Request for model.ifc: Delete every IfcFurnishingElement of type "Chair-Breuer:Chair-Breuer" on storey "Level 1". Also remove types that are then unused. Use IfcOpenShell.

First a look at what the model holds.

```python
import ifcopenshell
import ifcopenshell.util.element

model = ifcopenshell.open("model.ifc")
print(model.schema)
storey = next(s for s in model.by_type("IfcBuildingStorey") if s.Name == "Level 1")
furniture = [e for e in ifcopenshell.util.element.get_decomposition(storey) if e.is_a("IfcFurnishingElement")]
seen = {}
for e in furniture:
    element_type = ifcopenshell.util.element.get_type(e)
    name = element_type.Name if element_type not in (None, e) else None
    seen[name] = seen.get(name, 0) + 1
for name, count in sorted(seen.items(), key=str):
    print(count, "x", name)
```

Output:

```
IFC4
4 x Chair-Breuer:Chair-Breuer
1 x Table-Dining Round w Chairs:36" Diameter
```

```python
import ifcopenshell
import ifcopenshell.api.root
import ifcopenshell.util.element

model = ifcopenshell.open("model.ifc")

storey = next(s for s in model.by_type("IfcBuildingStorey") if s.Name == "Level 1")
furniture = [e for e in ifcopenshell.util.element.get_decomposition(storey) if e.is_a("IfcFurnishingElement")]
targets = [e for e in furniture if (t := ifcopenshell.util.element.get_type(e)) not in (None, e) and t.Name == "Chair-Breuer:Chair-Breuer"]
types = {ifcopenshell.util.element.get_type(e) for e in targets} - {None, *targets}

for e in targets:
    ifcopenshell.api.root.remove_product(model, product=e)
print(len(targets), "removed")

unused = [t for t in types if not ifcopenshell.util.element.get_types(t)]
for t in unused:
    ifcopenshell.api.root.remove_product(model, product=t)
print(len(unused), "unused types removed")

model.write("model_v2.ifc")
```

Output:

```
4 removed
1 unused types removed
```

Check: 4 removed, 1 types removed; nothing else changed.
